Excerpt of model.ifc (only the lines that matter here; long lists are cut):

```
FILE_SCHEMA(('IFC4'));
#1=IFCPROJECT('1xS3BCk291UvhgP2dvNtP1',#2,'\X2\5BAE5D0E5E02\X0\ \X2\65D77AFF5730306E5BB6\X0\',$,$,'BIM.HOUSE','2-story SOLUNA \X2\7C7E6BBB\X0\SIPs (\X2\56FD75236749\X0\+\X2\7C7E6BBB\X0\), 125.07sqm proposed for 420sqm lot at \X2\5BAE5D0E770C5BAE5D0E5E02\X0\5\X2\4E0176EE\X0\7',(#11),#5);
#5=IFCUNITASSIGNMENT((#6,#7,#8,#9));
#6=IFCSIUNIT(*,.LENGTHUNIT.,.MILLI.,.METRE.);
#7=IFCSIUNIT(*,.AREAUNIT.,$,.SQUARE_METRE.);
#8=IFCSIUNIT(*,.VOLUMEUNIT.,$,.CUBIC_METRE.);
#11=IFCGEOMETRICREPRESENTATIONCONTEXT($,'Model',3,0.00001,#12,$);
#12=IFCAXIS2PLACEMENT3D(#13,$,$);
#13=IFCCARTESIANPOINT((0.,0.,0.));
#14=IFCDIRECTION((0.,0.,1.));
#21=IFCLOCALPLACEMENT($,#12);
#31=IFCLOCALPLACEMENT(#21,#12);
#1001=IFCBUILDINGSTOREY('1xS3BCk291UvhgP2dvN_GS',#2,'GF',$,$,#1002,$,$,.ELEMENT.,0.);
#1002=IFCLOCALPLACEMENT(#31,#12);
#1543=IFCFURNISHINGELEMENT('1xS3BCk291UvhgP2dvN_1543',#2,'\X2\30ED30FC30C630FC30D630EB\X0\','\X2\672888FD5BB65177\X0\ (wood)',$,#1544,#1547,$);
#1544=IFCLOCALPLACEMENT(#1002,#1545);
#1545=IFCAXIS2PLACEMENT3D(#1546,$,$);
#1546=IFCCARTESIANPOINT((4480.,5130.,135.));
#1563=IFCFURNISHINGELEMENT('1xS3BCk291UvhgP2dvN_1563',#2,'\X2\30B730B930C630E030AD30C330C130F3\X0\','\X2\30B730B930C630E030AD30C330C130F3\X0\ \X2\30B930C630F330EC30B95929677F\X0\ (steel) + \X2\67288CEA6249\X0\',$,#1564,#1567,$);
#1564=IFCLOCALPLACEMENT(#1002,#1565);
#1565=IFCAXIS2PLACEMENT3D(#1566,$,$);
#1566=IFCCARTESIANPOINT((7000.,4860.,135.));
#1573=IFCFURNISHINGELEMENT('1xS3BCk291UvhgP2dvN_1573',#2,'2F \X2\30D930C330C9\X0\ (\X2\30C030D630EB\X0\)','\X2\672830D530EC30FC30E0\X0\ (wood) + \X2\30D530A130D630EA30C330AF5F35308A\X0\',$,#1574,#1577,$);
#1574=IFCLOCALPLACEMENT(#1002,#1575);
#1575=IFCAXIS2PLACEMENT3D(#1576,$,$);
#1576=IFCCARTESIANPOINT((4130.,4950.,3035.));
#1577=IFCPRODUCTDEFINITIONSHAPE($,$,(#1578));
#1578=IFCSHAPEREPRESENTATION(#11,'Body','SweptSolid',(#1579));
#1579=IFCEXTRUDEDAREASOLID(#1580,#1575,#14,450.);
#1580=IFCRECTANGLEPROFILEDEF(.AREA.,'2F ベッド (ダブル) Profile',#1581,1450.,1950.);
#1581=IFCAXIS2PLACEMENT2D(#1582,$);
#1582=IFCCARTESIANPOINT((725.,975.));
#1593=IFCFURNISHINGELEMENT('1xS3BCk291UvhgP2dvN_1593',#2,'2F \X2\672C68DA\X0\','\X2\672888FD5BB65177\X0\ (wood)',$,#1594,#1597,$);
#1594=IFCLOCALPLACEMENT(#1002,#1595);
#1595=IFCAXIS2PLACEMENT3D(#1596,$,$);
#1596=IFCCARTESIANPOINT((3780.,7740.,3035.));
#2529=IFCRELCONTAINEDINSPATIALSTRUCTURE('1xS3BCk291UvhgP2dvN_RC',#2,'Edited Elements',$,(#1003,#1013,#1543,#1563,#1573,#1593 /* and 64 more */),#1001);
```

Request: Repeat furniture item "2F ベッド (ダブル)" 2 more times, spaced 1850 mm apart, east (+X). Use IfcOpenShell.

```python
import numpy as np
import ifcopenshell
import ifcopenshell.api.geometry
import ifcopenshell.api.root
import ifcopenshell.util.element
import ifcopenshell.util.placement
import ifcopenshell.util.unit

model = ifcopenshell.open("model.ifc")
unit_scale = ifcopenshell.util.unit.calculate_unit_scale(model)


def reuse_history(source, copy):
    """copy_class also copies each property set's owner history, people and application; keep the originals."""
    for rel in copy.IsDefinedBy:
        if rel.is_a("IfcRelDefinesByProperties") and (history := rel.RelatingPropertyDefinition.OwnerHistory):
            rel.RelatingPropertyDefinition.OwnerHistory = source.OwnerHistory
            ifcopenshell.util.element.remove_deep2(model, history)


source = model.by_guid("1xS3BCk291UvhgP2dvN_1573")
base = ifcopenshell.util.placement.get_local_placement(source.ObjectPlacement)
step = np.array([1.0, 0.0, 0.0]) * 1.85 / unit_scale

for i in range(1, 3):
    copy = ifcopenshell.api.root.copy_class(model, product=source)
    copy.Representation = ifcopenshell.util.element.copy_deep(
        model, source.Representation, exclude=["IfcGeometricRepresentationContext", "IfcRepresentationMap"]
    )
    reuse_history(source, copy)
    matrix = base.copy()
    matrix[:3, 3] += i * step
    print("added at", matrix[:3, 3].round(3) + 0.0)
    ifcopenshell.api.geometry.edit_object_placement(model, product=copy, matrix=matrix, is_si=False)

model.write("model-out.ifc")
```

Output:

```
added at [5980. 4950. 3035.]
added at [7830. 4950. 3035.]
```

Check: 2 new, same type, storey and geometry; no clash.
